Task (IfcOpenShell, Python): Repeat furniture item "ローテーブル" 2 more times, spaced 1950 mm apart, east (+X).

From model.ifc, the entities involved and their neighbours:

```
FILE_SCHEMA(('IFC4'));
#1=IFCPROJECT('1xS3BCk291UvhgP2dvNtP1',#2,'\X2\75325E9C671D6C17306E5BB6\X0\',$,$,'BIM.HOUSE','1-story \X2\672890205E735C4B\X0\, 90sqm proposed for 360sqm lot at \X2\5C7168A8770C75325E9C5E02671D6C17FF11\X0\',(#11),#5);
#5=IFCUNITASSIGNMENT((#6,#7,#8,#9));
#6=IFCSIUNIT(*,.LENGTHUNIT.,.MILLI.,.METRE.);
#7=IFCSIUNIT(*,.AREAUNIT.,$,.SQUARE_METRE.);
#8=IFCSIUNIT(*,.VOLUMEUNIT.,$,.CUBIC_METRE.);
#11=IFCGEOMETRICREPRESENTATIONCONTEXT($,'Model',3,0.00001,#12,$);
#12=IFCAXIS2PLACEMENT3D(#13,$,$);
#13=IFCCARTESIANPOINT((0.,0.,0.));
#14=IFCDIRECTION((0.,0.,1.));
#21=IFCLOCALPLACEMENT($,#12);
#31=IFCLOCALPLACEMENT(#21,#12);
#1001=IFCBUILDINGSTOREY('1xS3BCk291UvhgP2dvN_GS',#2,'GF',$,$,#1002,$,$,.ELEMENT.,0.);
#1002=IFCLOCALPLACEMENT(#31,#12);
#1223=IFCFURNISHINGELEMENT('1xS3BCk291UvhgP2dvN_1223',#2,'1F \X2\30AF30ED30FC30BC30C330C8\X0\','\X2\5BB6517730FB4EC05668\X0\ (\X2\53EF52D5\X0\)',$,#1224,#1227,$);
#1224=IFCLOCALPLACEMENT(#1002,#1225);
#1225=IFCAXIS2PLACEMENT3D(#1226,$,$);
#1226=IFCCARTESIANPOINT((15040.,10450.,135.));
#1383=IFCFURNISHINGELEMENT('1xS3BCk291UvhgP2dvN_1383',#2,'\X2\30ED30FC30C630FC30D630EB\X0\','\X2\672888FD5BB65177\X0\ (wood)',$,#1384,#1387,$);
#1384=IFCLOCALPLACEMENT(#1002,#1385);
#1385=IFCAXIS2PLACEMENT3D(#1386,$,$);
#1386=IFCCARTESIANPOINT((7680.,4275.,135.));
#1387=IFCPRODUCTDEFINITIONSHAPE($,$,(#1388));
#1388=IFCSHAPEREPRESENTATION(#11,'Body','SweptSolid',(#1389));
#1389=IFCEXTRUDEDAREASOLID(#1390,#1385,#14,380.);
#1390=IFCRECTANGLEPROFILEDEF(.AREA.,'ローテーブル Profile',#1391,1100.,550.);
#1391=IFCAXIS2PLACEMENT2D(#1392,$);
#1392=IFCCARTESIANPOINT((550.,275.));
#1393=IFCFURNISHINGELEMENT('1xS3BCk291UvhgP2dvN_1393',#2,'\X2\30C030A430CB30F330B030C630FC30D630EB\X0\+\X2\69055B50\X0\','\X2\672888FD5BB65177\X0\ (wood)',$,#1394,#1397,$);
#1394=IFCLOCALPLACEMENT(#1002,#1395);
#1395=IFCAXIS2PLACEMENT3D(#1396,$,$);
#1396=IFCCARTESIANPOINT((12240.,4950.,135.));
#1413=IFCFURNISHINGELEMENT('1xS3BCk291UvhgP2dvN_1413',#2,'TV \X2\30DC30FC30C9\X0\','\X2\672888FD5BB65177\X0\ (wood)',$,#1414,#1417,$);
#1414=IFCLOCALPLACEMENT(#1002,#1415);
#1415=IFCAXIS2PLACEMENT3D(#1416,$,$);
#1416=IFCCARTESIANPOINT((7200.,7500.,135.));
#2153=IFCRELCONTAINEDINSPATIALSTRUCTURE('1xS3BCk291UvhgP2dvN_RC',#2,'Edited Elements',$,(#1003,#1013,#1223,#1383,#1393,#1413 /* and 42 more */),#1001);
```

```python
import numpy as np
import ifcopenshell
import ifcopenshell.api.geometry
import ifcopenshell.api.root
import ifcopenshell.util.element
import ifcopenshell.util.placement

model = ifcopenshell.open("model.ifc")


def reuse_history(source, copy):
    """copy_class also copies each property set's owner history, people and application; keep the originals."""
    for rel in copy.IsDefinedBy:
        if rel.is_a("IfcRelDefinesByProperties") and (history := rel.RelatingPropertyDefinition.OwnerHistory):
            rel.RelatingPropertyDefinition.OwnerHistory = source.OwnerHistory
            ifcopenshell.util.element.remove_deep2(model, history)


source = model.by_guid("1xS3BCk291UvhgP2dvN_1383")
base = ifcopenshell.util.placement.get_local_placement(source.ObjectPlacement)
step = np.array([1.0, 0.0, 0.0]) * 1950.0

for i in range(1, 3):
    copy = ifcopenshell.api.root.copy_class(model, product=source)
    copy.Representation = ifcopenshell.util.element.copy_deep(
        model, source.Representation, exclude=["IfcGeometricRepresentationContext", "IfcRepresentationMap"]
    )
    reuse_history(source, copy)
    matrix = base.copy()
    matrix[:3, 3] += i * step
    print("added at", matrix[:3, 3].round(3) + 0.0)
    ifcopenshell.api.geometry.edit_object_placement(model, product=copy, matrix=matrix, is_si=False)

model.write("model_v2.ifc")
```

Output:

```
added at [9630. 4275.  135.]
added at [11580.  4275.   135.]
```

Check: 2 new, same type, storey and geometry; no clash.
